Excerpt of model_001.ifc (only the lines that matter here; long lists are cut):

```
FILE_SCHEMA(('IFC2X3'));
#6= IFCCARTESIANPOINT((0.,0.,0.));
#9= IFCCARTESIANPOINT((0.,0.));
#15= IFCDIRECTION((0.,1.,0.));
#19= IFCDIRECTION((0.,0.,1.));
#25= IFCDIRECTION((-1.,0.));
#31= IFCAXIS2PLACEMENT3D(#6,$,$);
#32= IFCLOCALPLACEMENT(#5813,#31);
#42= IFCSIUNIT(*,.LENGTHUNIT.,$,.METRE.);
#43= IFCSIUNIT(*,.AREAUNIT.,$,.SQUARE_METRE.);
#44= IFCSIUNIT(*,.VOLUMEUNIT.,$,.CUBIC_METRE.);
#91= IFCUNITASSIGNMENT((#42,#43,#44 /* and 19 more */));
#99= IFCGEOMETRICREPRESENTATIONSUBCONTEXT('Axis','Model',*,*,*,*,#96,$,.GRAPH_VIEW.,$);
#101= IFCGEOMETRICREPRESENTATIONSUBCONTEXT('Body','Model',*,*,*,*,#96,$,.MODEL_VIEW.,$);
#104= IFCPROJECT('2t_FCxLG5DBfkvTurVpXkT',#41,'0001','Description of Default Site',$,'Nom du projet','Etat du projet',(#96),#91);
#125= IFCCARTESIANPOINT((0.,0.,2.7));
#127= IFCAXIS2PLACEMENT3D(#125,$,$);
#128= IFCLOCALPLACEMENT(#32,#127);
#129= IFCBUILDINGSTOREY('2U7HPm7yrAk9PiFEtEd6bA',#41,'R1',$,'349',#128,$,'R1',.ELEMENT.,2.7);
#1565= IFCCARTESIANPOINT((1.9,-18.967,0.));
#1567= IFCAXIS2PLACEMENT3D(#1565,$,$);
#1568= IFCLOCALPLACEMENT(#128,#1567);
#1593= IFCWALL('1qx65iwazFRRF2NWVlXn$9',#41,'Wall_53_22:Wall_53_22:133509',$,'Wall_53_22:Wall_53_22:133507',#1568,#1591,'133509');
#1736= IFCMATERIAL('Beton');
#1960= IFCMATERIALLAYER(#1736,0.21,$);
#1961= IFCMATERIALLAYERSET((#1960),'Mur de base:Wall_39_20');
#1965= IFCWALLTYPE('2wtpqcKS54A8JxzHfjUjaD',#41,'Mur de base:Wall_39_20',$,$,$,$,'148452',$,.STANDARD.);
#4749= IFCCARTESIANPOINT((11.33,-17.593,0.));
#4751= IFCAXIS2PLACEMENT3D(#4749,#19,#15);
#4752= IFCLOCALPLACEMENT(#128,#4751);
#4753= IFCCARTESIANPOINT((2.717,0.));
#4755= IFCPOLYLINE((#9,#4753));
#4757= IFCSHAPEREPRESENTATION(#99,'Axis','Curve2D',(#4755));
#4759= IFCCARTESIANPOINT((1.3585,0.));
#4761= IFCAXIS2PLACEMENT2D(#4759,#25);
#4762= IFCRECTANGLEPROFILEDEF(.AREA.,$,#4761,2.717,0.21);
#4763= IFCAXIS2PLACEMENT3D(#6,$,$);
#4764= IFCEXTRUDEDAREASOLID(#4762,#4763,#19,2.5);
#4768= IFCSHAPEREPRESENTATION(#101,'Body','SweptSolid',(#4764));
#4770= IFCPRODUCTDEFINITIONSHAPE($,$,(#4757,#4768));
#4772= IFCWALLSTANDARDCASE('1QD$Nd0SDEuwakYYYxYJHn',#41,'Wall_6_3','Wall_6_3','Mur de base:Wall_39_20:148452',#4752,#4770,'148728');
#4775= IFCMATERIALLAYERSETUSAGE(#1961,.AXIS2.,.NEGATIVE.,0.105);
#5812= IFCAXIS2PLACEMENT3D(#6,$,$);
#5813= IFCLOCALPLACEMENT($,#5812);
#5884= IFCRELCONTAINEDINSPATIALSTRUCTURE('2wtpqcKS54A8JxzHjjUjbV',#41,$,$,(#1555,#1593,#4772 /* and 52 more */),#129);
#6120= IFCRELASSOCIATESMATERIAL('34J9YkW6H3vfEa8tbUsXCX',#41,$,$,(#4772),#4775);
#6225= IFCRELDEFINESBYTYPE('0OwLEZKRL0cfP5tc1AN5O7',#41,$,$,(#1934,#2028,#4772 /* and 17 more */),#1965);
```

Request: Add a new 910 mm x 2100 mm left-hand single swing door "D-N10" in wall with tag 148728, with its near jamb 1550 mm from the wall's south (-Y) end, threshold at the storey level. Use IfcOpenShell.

```python
import numpy as np
import ifcopenshell
import ifcopenshell.api.feature
import ifcopenshell.api.geometry
import ifcopenshell.api.root
import ifcopenshell.api.spatial
import ifcopenshell.api.type
import ifcopenshell.geom
import ifcopenshell.util.element
import ifcopenshell.util.placement
import ifcopenshell.util.representation
import ifcopenshell.util.shape
import ifcopenshell.util.unit

model = ifcopenshell.open("model_001.ifc")
unit_scale = ifcopenshell.util.unit.calculate_unit_scale(model)
settings = ifcopenshell.geom.settings()


def volume(element):
    """Net volume in cubic metres, openings subtracted."""
    shape = ifcopenshell.geom.create_shape(settings, element)
    return ifcopenshell.util.shape.get_volume(shape.geometry)


wall = model.by_guid("1QD$Nd0SDEuwakYYYxYJHn")
storey = ifcopenshell.util.element.get_container(wall, ifc_class="IfcBuildingStorey")
context = ifcopenshell.util.representation.get_context(model, "Model", "Body", "MODEL_VIEW")
before = volume(wall)

width, height, from_end, sill = 0.91, 2.1, 1.55, 0.0  # metres

# The wall runs along its own X axis, and the end named is its -X end.
wall_shape = ifcopenshell.geom.create_shape(settings, wall)
x, y, z = ifcopenshell.util.shape.get_vertices(wall_shape.geometry).T
start = x.min() + from_end
face, thickness = float(y.min()), float(y.max() - y.min())
wall_matrix = ifcopenshell.util.placement.get_local_placement(wall.ObjectPlacement)
level = ifcopenshell.util.placement.get_local_placement(storey.ObjectPlacement)[2, 3]


def in_wall(x, y):
    """Placement at x, y metres in the wall's axes, at sill height."""
    matrix = wall_matrix.copy()
    matrix[:, 3] = wall_matrix @ np.array([x / unit_scale, y / unit_scale, 0.0, 1.0])
    matrix[2, 3] = level + sill / unit_scale
    return matrix


# Opening: a box that overshoots both wall faces by 50 mm.
opening = ifcopenshell.api.root.create_entity(model, ifc_class="IfcOpeningElement")
box = ifcopenshell.api.geometry.add_wall_representation(
    model, context=context, length=width, height=height, thickness=thickness + 0.1
)
ifcopenshell.api.geometry.assign_representation(model, product=opening, representation=box)
ifcopenshell.api.geometry.edit_object_placement(model, product=opening, matrix=in_wall(start, face - 0.05), is_si=False)
ifcopenshell.api.feature.add_feature(model, feature=opening, element=wall)

door = ifcopenshell.api.root.create_entity(model, ifc_class="IfcDoor", name="D-N10")
door.OverallWidth, door.OverallHeight = width / unit_scale, height / unit_scale
body = ifcopenshell.api.geometry.add_door_representation(
    model,
    context=context,
    overall_width=door.OverallWidth,
    overall_height=door.OverallHeight,
    operation_type="SINGLE_SWING_LEFT",
    lining_properties={"LiningDepth": thickness / unit_scale, "ThresholdDepth": thickness / unit_scale},
)
ifcopenshell.api.geometry.assign_representation(model, product=door, representation=body)
ifcopenshell.api.spatial.assign_container(model, products=[door], relating_structure=storey)
fills = ifcopenshell.api.feature.add_filling(model, opening=opening, element=door)
fills.OwnerHistory = door.OwnerHistory  # required in IFC2X3

# IFC2X3 keeps the operation on the door style.
style = ifcopenshell.api.root.create_entity(model, ifc_class="IfcDoorStyle", name="D-N10")
style.OperationType, style.ConstructionType = "SINGLE_SWING_LEFT", "NOTDEFINED"
style.ParameterTakesPrecedence = style.Sizeable = False
ifcopenshell.api.type.assign_type(model, related_objects=[door], relating_type=style)

# The lining spans the wall, so the door starts at the wall face.
ifcopenshell.api.geometry.edit_object_placement(model, product=door, matrix=in_wall(start, face), is_si=False)

after = volume(wall)

print(f"wall volume {before:.3f} -> {after:.3f} m3")

model.write("model_001_rev.ifc")
```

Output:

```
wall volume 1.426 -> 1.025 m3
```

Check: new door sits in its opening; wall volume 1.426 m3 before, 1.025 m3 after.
